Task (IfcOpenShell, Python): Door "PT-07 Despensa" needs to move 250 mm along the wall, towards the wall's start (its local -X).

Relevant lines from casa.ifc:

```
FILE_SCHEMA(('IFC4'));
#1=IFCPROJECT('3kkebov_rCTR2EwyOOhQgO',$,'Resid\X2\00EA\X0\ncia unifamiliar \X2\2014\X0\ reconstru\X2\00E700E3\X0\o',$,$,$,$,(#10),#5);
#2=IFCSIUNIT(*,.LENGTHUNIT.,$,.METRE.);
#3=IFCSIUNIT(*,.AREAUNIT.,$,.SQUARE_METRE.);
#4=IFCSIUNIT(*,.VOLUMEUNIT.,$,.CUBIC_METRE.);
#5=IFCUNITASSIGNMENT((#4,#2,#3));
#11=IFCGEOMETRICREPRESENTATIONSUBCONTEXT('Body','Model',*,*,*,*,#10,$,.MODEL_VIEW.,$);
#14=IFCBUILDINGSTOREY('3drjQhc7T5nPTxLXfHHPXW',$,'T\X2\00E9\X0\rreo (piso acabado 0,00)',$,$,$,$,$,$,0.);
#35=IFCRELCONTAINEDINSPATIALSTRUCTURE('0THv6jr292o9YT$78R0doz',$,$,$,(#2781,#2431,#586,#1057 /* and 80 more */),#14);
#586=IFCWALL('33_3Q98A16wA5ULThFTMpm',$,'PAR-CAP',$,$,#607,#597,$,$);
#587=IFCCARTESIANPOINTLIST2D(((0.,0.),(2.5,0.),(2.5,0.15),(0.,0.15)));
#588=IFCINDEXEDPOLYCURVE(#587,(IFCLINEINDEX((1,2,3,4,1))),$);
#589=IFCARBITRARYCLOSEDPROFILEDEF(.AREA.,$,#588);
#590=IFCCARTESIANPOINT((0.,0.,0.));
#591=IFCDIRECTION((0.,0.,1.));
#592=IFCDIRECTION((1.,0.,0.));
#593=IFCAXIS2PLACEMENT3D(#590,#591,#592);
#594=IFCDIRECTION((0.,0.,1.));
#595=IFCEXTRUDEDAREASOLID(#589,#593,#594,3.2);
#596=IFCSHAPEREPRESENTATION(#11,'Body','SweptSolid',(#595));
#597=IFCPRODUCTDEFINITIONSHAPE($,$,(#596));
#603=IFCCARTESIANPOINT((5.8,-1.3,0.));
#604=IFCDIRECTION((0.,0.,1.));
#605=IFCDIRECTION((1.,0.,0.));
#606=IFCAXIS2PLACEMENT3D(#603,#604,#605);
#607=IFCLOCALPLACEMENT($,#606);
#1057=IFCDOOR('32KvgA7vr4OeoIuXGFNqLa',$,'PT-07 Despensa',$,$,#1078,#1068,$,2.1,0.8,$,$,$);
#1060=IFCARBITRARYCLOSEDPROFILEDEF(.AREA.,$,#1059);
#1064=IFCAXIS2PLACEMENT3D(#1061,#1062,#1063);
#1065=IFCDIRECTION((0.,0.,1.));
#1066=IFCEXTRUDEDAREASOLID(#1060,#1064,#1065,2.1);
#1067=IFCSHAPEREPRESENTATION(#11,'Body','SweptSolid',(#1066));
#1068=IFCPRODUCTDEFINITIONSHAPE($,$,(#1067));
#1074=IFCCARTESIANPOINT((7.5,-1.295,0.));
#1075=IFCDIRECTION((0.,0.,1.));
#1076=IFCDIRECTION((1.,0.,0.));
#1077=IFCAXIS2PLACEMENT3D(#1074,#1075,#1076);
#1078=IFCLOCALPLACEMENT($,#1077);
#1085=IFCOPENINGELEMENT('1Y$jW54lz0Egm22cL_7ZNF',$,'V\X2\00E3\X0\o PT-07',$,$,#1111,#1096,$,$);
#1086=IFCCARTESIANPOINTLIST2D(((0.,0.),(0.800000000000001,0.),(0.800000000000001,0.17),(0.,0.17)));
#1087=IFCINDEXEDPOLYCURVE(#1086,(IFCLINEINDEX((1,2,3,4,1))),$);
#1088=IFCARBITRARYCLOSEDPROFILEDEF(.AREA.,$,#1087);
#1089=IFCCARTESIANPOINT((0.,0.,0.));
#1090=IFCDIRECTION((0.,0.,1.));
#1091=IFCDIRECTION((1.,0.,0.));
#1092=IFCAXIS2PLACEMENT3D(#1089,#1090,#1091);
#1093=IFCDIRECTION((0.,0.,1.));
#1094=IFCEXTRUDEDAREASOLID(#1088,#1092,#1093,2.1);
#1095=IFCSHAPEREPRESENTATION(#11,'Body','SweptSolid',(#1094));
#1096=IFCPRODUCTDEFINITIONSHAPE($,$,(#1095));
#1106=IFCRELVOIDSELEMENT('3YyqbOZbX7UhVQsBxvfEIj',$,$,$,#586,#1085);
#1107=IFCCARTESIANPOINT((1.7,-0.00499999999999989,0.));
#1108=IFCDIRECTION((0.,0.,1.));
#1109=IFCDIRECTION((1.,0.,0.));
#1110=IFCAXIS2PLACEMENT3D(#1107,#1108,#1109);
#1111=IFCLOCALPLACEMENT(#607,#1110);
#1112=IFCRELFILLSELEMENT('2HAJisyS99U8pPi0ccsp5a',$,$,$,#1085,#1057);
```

```python
import ifcopenshell
import ifcopenshell.api.geometry
import ifcopenshell.util.placement
import ifcopenshell.util.unit

model = ifcopenshell.open("casa.ifc")
unit_scale = ifcopenshell.util.unit.calculate_unit_scale(model)

door = model.by_guid("32KvgA7vr4OeoIuXGFNqLa")
opening = door.FillsVoids[0].RelatingOpeningElement
wall = opening.VoidsElements[0].RelatingBuildingElement

wall_matrix = ifcopenshell.util.placement.get_local_placement(wall.ObjectPlacement)
shift = wall_matrix[:3, 0] * -0.25 / unit_scale
before = ifcopenshell.util.placement.get_local_placement(door.ObjectPlacement)[:3, 3].copy()

# The door is not placed relative to its opening, so move both.
for product in (opening, door):
    matrix = ifcopenshell.util.placement.get_local_placement(product.ObjectPlacement)
    matrix[:3, 3] += shift
    ifcopenshell.api.geometry.edit_object_placement(model, product=product, matrix=matrix, is_si=False)

after = ifcopenshell.util.placement.get_local_placement(door.ObjectPlacement)[:3, 3]
print("door moved by", (after - before).round(3) + 0.0)

model.write("casa_updated.ifc")
```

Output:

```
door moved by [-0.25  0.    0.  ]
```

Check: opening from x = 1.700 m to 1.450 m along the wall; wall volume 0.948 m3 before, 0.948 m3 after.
